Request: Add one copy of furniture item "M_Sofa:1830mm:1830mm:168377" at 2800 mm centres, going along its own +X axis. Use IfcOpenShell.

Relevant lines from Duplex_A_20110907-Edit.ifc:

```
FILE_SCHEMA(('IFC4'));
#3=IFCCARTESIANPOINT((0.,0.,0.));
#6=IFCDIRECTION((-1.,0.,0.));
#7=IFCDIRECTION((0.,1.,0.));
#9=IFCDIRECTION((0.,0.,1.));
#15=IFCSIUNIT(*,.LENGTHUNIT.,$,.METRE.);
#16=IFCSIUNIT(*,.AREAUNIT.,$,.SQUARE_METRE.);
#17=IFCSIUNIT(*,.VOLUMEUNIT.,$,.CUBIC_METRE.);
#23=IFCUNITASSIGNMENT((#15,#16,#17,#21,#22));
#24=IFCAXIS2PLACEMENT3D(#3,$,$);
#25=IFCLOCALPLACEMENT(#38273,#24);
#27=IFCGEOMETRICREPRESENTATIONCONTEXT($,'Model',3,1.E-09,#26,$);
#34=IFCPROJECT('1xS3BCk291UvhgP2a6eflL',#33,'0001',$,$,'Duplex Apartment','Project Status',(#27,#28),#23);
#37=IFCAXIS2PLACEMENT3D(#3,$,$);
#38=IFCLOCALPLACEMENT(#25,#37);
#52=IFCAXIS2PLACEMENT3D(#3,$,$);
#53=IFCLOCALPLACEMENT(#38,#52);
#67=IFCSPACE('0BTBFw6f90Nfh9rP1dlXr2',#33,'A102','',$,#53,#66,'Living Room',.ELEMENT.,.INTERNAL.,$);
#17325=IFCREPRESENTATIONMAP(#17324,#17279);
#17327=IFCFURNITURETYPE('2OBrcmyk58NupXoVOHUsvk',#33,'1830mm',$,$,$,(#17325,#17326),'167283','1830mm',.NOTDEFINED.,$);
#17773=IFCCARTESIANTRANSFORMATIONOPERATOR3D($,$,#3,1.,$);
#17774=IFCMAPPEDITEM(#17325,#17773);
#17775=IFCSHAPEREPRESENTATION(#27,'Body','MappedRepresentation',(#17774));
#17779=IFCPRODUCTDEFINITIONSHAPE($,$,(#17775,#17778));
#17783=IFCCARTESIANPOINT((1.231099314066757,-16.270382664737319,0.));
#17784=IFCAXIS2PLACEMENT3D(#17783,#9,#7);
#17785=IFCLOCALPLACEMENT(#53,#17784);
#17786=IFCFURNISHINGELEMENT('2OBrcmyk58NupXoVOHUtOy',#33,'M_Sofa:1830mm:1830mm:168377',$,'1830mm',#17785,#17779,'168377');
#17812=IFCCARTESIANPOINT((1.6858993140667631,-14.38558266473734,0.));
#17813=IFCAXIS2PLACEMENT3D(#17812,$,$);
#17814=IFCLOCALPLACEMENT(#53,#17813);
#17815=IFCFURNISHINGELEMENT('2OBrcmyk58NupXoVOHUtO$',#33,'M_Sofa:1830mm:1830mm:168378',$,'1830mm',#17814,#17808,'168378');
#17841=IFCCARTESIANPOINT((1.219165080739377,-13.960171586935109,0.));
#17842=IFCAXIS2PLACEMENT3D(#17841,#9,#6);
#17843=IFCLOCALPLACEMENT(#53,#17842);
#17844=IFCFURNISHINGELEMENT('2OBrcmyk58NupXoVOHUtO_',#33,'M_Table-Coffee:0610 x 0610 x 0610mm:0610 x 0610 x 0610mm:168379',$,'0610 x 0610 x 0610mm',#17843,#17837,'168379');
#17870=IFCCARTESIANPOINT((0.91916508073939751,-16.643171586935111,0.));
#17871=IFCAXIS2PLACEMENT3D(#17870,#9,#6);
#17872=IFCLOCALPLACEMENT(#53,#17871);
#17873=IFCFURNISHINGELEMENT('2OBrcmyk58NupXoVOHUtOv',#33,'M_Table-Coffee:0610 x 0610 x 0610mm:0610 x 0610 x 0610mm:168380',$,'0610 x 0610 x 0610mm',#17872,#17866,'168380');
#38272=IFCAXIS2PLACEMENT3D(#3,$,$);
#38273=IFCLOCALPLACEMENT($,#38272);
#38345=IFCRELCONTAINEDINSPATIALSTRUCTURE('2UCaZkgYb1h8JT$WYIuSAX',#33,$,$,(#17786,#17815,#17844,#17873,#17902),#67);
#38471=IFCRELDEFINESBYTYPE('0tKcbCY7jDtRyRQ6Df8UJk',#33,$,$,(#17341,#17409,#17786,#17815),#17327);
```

```python
import ifcopenshell
import ifcopenshell.api.geometry
import ifcopenshell.api.root
import ifcopenshell.util.element
import ifcopenshell.util.placement
import ifcopenshell.util.unit

model = ifcopenshell.open("Duplex_A_20110907-Edit.ifc")
unit_scale = ifcopenshell.util.unit.calculate_unit_scale(model)


def reuse_history(source, copy):
    """copy_class also copies each property set's owner history, people and application; keep the originals."""
    for rel in copy.IsDefinedBy:
        if rel.is_a("IfcRelDefinesByProperties") and (history := rel.RelatingPropertyDefinition.OwnerHistory):
            rel.RelatingPropertyDefinition.OwnerHistory = source.OwnerHistory
            ifcopenshell.util.element.remove_deep2(model, history)


source = model.by_id(17786)
base = ifcopenshell.util.placement.get_local_placement(source.ObjectPlacement)
step = base[:3, 0] * 2.8 / unit_scale

for i in range(1, 2):
    copy = ifcopenshell.api.root.copy_class(model, product=source)
    copy.Representation = ifcopenshell.util.element.copy_deep(
        model, source.Representation, exclude=["IfcGeometricRepresentationContext", "IfcRepresentationMap"]
    )
    copy.Name = "M_Sofa:1830mm:1830mm"
    copy.Tag = None
    reuse_history(source, copy)
    matrix = base.copy()
    matrix[:3, 3] += i * step
    print("added at", matrix[:3, 3].round(3) + 0.0)
    ifcopenshell.api.geometry.edit_object_placement(model, product=copy, matrix=matrix, is_si=False)

model.write("Duplex_A_20110907-Edit-out.ifc")
```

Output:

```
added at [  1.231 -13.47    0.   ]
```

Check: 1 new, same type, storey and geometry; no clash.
